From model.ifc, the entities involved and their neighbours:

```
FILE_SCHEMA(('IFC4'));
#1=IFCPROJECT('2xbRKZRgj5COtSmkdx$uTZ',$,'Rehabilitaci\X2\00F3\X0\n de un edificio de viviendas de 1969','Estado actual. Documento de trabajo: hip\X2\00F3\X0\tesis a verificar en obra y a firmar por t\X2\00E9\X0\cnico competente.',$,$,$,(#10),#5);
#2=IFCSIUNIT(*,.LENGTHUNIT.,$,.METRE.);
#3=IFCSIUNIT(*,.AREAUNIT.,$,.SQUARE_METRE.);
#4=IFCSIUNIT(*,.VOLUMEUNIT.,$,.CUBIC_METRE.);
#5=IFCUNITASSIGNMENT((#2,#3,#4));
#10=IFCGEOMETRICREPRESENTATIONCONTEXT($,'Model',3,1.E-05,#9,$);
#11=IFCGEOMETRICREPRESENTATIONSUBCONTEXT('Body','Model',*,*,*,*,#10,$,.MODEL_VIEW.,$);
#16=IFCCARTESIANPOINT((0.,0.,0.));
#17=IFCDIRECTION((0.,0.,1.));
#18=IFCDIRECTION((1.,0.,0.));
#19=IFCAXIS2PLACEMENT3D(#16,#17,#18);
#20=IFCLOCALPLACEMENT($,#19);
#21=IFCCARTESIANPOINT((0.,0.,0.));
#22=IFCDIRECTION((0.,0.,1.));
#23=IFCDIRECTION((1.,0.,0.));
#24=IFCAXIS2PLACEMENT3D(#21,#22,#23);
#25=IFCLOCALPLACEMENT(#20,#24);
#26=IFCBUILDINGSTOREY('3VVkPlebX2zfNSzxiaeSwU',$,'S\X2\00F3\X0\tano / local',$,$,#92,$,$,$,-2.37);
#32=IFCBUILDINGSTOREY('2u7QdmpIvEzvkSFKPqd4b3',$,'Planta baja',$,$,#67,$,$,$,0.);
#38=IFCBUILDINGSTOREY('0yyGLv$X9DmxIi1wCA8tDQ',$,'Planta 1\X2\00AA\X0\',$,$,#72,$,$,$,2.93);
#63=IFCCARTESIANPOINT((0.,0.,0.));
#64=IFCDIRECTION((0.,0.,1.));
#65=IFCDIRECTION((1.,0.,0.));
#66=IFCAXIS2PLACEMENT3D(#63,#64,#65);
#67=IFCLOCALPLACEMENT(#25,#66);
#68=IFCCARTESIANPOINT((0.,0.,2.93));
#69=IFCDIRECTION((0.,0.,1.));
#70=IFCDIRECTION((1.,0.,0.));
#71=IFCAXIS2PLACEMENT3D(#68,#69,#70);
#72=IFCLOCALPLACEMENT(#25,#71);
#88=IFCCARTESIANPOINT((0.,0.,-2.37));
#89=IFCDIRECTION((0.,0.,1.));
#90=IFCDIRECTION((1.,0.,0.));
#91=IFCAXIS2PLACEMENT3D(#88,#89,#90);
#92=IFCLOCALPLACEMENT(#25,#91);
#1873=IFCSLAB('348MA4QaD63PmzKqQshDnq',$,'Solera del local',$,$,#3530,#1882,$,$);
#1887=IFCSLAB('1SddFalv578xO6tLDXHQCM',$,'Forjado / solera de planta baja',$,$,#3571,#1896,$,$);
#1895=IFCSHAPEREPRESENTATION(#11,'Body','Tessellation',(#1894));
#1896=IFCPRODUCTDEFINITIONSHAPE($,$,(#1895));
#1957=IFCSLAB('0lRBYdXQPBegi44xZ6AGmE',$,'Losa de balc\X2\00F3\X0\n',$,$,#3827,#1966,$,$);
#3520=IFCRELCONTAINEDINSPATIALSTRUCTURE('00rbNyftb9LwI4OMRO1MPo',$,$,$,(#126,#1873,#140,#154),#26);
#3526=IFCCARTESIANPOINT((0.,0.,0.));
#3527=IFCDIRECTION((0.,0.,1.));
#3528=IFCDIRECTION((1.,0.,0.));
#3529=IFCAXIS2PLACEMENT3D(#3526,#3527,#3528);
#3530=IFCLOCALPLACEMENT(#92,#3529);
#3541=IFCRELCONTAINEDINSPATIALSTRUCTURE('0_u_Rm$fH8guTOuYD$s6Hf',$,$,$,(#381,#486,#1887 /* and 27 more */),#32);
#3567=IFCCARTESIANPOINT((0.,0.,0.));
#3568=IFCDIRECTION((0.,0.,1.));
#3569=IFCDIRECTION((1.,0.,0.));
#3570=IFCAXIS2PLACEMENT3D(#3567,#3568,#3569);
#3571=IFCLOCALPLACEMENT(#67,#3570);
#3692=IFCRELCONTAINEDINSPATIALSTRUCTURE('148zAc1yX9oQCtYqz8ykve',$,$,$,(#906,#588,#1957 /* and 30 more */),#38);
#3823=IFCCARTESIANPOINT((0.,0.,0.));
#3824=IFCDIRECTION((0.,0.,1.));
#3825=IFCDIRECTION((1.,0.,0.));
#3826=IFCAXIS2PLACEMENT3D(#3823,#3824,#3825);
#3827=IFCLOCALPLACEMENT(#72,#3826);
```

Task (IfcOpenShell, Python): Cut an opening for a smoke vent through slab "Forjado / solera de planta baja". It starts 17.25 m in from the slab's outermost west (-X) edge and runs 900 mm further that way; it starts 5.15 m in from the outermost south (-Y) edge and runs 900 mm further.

```python
import numpy as np
import ifcopenshell
import ifcopenshell.api.feature
import ifcopenshell.api.geometry
import ifcopenshell.api.root
import ifcopenshell.geom
import ifcopenshell.util.placement
import ifcopenshell.util.representation
import ifcopenshell.util.shape
import ifcopenshell.util.unit

model = ifcopenshell.open("model.ifc")
unit_scale = ifcopenshell.util.unit.calculate_unit_scale(model)
settings = ifcopenshell.geom.settings()


def volume(element):
    """Net volume in cubic metres, openings subtracted."""
    shape = ifcopenshell.geom.create_shape(settings, element)
    return ifcopenshell.util.shape.get_volume(shape.geometry)


slab = model.by_guid("1SddFalv578xO6tLDXHQCM")
before = volume(slab)

# Extent in the slab's own axes, in metres. The edges named are its -X and -Y sides.
slab_shape = ifcopenshell.geom.create_shape(settings, slab)
vertices = ifcopenshell.util.shape.get_vertices(slab_shape.geometry)
x_min, y_min, bottom = vertices.min(axis=0)
top = vertices[:, 2].max()

opening = ifcopenshell.api.root.create_entity(model, ifc_class="IfcOpeningElement", name="Smoke vent opening", predefined_type="OPENING")
context = ifcopenshell.util.representation.get_context(model, "Model", "Body", "MODEL_VIEW")
width, depth = 0.9, 0.9
outline = [(0.0, 0.0), (width, 0.0), (width, depth), (0.0, depth), (0.0, 0.0)]
# Overshoot both faces by 50 mm so the cut is clean.
shape = ifcopenshell.api.geometry.add_slab_representation(
    model, context=context, depth=top - bottom + 0.1, polyline=outline
)
ifcopenshell.api.geometry.assign_representation(model, product=opening, representation=shape)

matrix = ifcopenshell.util.placement.get_local_placement(slab.ObjectPlacement)
matrix[:, 3] = matrix @ np.append(np.array([x_min + 17.25, y_min + 5.15, bottom - 0.05]) / unit_scale, 1.0)
ifcopenshell.api.geometry.edit_object_placement(model, product=opening, matrix=matrix, is_si=False)
ifcopenshell.api.feature.add_feature(model, feature=opening, element=slab)

after = volume(slab)

print(f"slab volume {before:.3f} -> {after:.3f} m3")

model.write("model_v2.ifc")
```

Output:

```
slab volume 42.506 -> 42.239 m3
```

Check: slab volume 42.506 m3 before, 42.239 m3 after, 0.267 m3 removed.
